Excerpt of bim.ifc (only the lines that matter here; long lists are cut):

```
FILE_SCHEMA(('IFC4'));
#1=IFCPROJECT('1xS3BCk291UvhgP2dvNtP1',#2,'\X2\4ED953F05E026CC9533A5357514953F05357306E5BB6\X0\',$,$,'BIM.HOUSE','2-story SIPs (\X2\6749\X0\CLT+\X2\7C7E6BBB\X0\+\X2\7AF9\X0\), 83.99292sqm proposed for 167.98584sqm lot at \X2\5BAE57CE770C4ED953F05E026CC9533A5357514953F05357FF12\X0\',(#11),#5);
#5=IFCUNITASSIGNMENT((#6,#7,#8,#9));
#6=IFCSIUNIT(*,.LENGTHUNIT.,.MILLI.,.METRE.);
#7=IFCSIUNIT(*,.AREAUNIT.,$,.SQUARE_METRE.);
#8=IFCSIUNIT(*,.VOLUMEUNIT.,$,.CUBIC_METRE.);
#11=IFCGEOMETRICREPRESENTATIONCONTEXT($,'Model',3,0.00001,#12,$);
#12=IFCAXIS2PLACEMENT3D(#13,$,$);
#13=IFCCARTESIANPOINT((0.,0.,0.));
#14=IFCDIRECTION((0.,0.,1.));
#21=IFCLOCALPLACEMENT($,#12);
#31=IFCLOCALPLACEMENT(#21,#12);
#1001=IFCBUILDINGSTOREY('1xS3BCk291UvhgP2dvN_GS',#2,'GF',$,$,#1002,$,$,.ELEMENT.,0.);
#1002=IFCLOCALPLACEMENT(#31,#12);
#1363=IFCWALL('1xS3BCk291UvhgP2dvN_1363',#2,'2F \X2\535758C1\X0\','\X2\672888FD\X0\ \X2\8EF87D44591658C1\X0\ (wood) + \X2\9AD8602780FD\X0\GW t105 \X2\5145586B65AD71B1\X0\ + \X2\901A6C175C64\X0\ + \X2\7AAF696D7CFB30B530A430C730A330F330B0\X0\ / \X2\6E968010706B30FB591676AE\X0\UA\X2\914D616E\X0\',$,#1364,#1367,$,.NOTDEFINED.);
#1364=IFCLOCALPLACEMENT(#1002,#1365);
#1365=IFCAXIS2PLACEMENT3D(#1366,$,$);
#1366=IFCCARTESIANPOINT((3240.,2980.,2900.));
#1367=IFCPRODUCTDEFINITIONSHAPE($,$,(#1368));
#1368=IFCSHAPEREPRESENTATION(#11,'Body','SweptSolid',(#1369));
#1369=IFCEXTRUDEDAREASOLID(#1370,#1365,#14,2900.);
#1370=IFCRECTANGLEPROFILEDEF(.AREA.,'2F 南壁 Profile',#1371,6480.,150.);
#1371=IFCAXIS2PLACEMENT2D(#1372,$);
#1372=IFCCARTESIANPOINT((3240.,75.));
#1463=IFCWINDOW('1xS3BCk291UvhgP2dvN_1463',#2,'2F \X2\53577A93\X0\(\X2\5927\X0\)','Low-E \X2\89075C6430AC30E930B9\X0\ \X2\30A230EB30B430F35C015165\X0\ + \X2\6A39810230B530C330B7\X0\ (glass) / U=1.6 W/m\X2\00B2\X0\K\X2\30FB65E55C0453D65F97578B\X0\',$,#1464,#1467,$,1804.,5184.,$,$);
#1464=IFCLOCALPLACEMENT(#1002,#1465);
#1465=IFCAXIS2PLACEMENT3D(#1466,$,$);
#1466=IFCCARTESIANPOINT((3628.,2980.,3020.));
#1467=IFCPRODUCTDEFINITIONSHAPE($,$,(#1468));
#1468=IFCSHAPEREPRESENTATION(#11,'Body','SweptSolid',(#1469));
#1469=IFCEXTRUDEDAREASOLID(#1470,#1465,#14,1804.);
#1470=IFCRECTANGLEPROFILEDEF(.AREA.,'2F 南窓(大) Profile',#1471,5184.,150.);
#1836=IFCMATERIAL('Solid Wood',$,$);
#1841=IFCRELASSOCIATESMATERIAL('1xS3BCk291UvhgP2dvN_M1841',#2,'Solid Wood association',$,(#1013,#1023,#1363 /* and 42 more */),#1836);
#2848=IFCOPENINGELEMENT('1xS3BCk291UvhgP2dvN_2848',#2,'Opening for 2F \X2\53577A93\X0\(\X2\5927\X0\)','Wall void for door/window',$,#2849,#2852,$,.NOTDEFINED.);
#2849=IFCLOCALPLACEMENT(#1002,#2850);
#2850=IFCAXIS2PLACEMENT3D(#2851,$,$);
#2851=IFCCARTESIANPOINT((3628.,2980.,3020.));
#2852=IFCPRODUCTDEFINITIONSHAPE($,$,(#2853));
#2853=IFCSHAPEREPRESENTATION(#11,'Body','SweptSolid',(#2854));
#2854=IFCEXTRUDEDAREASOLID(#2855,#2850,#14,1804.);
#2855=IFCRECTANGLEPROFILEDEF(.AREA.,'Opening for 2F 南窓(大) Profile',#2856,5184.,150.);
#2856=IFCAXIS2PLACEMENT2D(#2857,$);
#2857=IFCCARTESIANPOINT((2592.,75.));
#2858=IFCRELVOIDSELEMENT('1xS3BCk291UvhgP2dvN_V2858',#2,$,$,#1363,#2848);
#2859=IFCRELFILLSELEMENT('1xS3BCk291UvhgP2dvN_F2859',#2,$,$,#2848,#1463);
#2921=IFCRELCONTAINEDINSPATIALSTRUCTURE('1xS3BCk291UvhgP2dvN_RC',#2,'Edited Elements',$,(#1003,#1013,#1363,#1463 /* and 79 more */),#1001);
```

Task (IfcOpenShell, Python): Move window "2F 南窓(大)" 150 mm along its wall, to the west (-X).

```python
import ifcopenshell
import ifcopenshell.api.geometry
import ifcopenshell.util.placement
import ifcopenshell.util.unit

model = ifcopenshell.open("bim.ifc")
unit_scale = ifcopenshell.util.unit.calculate_unit_scale(model)

window = model.by_id(1463)
opening = window.FillsVoids[0].RelatingOpeningElement
wall = opening.VoidsElements[0].RelatingBuildingElement

wall_matrix = ifcopenshell.util.placement.get_local_placement(wall.ObjectPlacement)
shift = wall_matrix[:3, 0] * -0.15 / unit_scale
before = ifcopenshell.util.placement.get_local_placement(window.ObjectPlacement)[:3, 3].copy()

# The window is not placed relative to its opening, so move both.
for product in (opening, window):
    matrix = ifcopenshell.util.placement.get_local_placement(product.ObjectPlacement)
    matrix[:3, 3] += shift
    ifcopenshell.api.geometry.edit_object_placement(model, product=product, matrix=matrix, is_si=False)

after = ifcopenshell.util.placement.get_local_placement(window.ObjectPlacement)[:3, 3]
print("window moved by", (after - before).round(3) + 0.0)

model.write("bim_v2.ifc")
```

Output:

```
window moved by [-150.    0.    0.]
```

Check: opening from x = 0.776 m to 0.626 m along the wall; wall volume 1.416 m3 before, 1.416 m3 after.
